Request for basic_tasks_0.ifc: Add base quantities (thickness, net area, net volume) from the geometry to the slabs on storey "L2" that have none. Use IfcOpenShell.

First a look at what the model holds.

```python
import ifcopenshell
import ifcopenshell.util.element
import ifcopenshell.util.unit

model = ifcopenshell.open("basic_tasks_0.ifc")
print(model.schema)
for unit_type in ("LENGTHUNIT", "AREAUNIT", "VOLUMEUNIT"):
    print(unit_type, ifcopenshell.util.unit.calculate_unit_scale(model, unit_type))
storey = next(s for s in model.by_type("IfcBuildingStorey") if s.Name == "L2")
slabs = [e for e in ifcopenshell.util.element.get_decomposition(storey) if e.is_a("IfcSlab")]
for e in sorted(slabs, key=lambda e: e.id()):
    print(e.id(), e.is_a(), e.Name, list(ifcopenshell.util.element.get_psets(e, qtos_only=True)), sep=" | ")
```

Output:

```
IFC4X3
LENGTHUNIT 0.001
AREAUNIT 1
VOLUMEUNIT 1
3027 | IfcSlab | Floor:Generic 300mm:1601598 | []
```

```python
import ifcopenshell
import ifcopenshell.api.pset
import ifcopenshell.geom
import ifcopenshell.util.element
import ifcopenshell.util.shape
import ifcopenshell.util.unit

model = ifcopenshell.open("basic_tasks_0.ifc")
unit_scale = ifcopenshell.util.unit.calculate_unit_scale(model)
area_scale = ifcopenshell.util.unit.calculate_unit_scale(model, "AREAUNIT")
volume_scale = ifcopenshell.util.unit.calculate_unit_scale(model, "VOLUMEUNIT")
settings = ifcopenshell.geom.settings()

storey = next(s for s in model.by_type("IfcBuildingStorey") if s.Name == "L2")
slabs = [e for e in ifcopenshell.util.element.get_decomposition(storey) if e.is_a("IfcSlab")]

for e in sorted(slabs, key=lambda e: e.id()):
    if ifcopenshell.util.element.get_psets(e, qtos_only=True, should_inherit=False):
        continue
    # Geometry comes back in metres, in the element's own axes.
    shape = ifcopenshell.geom.create_shape(settings, e)
    values = {
        "Width": ifcopenshell.util.shape.get_z(shape.geometry) / unit_scale,
        "NetArea": ifcopenshell.util.shape.get_footprint_area(shape.geometry) / area_scale,
        "NetVolume": ifcopenshell.util.shape.get_volume(shape.geometry) / volume_scale,
    }
    qto = ifcopenshell.api.pset.add_qto(model, product=e, name="Qto_SlabBaseQuantities")
    ifcopenshell.api.pset.edit_qto(model, qto=qto, properties=values)
    print(e.id(), {k: round(v, 3) for k, v in values.items()})

model.write("basic_tasks_0-out.ifc")
```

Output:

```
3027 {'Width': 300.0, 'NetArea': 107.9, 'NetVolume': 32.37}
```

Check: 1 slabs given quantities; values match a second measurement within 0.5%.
